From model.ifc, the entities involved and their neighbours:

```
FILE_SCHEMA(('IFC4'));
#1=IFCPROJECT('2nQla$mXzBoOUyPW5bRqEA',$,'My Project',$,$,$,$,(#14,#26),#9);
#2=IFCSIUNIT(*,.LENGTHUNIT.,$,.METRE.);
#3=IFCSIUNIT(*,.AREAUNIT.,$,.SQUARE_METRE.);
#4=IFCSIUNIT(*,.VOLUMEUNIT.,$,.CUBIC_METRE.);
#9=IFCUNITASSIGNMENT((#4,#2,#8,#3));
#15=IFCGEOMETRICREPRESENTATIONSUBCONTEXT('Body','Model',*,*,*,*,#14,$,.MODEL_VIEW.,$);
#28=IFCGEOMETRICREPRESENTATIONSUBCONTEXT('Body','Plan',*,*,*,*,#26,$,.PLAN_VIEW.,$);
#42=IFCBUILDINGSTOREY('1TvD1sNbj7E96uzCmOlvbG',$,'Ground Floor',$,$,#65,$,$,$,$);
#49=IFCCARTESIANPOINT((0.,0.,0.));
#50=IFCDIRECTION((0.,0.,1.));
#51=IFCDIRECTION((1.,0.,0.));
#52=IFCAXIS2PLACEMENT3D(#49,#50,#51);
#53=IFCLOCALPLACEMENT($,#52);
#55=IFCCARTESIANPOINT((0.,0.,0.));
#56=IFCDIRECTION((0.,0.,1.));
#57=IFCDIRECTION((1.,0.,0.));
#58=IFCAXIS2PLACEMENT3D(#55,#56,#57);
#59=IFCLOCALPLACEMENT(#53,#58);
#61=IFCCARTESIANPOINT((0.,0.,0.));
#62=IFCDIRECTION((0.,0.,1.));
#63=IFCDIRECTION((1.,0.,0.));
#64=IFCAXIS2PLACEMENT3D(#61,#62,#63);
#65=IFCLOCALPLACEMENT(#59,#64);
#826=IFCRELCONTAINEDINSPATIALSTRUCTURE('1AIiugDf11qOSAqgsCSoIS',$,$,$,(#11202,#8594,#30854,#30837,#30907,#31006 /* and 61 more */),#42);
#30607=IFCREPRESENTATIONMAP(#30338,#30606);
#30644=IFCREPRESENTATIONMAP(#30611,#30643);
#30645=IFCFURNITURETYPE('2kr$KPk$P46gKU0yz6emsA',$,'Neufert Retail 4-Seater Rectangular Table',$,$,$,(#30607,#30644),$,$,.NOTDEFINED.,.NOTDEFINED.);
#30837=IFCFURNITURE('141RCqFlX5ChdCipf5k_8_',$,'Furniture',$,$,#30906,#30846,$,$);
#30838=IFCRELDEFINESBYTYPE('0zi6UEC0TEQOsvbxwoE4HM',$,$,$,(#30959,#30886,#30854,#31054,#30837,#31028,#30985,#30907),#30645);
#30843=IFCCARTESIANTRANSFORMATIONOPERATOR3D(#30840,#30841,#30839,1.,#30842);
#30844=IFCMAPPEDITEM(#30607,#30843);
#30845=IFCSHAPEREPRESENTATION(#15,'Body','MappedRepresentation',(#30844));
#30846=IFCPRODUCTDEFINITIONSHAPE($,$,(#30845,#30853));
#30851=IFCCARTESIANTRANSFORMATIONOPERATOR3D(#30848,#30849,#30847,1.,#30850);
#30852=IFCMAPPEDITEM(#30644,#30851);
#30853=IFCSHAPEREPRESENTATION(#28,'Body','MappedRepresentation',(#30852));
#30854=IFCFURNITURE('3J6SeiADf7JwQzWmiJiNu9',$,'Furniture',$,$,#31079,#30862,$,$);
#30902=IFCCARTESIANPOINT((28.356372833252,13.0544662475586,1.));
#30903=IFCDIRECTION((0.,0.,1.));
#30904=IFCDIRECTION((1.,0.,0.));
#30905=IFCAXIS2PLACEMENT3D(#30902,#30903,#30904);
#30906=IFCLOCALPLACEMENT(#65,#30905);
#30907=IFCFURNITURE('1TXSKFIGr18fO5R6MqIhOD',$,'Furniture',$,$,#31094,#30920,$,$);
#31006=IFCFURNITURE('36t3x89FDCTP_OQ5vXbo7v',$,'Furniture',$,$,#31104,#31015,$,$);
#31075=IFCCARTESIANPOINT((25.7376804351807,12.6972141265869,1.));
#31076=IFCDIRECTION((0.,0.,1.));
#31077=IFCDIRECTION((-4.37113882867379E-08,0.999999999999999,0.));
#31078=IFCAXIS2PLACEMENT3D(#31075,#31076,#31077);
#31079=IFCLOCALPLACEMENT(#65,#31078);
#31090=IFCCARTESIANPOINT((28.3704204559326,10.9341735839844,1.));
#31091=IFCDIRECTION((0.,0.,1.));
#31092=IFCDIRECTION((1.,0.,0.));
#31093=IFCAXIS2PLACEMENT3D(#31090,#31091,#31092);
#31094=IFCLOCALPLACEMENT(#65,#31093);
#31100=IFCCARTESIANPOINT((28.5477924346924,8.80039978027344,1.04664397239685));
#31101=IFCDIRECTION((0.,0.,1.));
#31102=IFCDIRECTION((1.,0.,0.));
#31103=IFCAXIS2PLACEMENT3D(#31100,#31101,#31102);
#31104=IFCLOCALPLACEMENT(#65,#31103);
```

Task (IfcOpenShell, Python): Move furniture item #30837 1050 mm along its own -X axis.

```python
import ifcopenshell
import ifcopenshell.api.geometry
import ifcopenshell.util.placement

model = ifcopenshell.open("model.ifc")

item = model.by_guid("141RCqFlX5ChdCipf5k_8_")
matrix = ifcopenshell.util.placement.get_local_placement(item.ObjectPlacement)
matrix[:3, 3] -= matrix[:3, 0] * 1.05
ifcopenshell.api.geometry.edit_object_placement(model, product=item, matrix=matrix, is_si=False)

print(ifcopenshell.util.placement.get_local_placement(item.ObjectPlacement).round(3) + 0.0)

model.write("model_edited.ifc")
```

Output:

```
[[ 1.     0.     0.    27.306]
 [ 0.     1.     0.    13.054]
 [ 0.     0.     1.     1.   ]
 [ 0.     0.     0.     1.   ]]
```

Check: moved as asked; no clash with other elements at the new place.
